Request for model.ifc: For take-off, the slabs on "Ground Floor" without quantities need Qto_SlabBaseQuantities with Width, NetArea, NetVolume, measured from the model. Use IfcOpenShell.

First a look at what the model holds.

```python
import ifcopenshell
import ifcopenshell.util.element
import ifcopenshell.util.unit

model = ifcopenshell.open("model.ifc")
print(model.schema)
for unit_type in ("LENGTHUNIT", "AREAUNIT", "VOLUMEUNIT"):
    print(unit_type, ifcopenshell.util.unit.calculate_unit_scale(model, unit_type))
storey = next(s for s in model.by_type("IfcBuildingStorey") if s.Name == "Ground Floor")
slabs = [e for e in ifcopenshell.util.element.get_decomposition(storey) if e.is_a("IfcSlab")]
for e in sorted(slabs, key=lambda e: e.id()):
    print(e.id(), e.is_a(), e.Name, list(ifcopenshell.util.element.get_psets(e, qtos_only=True)), sep=" | ")
```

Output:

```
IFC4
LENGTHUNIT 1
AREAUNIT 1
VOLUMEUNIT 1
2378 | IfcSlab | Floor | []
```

```python
import ifcopenshell
import ifcopenshell.api.pset
import ifcopenshell.geom
import ifcopenshell.util.element
import ifcopenshell.util.shape
import ifcopenshell.util.unit

model = ifcopenshell.open("model.ifc")
unit_scale = ifcopenshell.util.unit.calculate_unit_scale(model)
area_scale = ifcopenshell.util.unit.calculate_unit_scale(model, "AREAUNIT")
volume_scale = ifcopenshell.util.unit.calculate_unit_scale(model, "VOLUMEUNIT")
settings = ifcopenshell.geom.settings()

storey = next(s for s in model.by_type("IfcBuildingStorey") if s.Name == "Ground Floor")
slabs = [e for e in ifcopenshell.util.element.get_decomposition(storey) if e.is_a("IfcSlab")]

for e in sorted(slabs, key=lambda e: e.id()):
    if ifcopenshell.util.element.get_psets(e, qtos_only=True, should_inherit=False):
        continue
    # Geometry comes back in metres, in the element's own axes.
    shape = ifcopenshell.geom.create_shape(settings, e)
    values = {
        "Width": ifcopenshell.util.shape.get_z(shape.geometry) / unit_scale,
        "NetArea": ifcopenshell.util.shape.get_footprint_area(shape.geometry) / area_scale,
        "NetVolume": ifcopenshell.util.shape.get_volume(shape.geometry) / volume_scale,
    }
    qto = ifcopenshell.api.pset.add_qto(model, product=e, name="Qto_SlabBaseQuantities")
    ifcopenshell.api.pset.edit_qto(model, qto=qto, properties=values)
    print(e.id(), {k: round(v, 3) for k, v in values.items()})

model.write("model_updated.ifc")
```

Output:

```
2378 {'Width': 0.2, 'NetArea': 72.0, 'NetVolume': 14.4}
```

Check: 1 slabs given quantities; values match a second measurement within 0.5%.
